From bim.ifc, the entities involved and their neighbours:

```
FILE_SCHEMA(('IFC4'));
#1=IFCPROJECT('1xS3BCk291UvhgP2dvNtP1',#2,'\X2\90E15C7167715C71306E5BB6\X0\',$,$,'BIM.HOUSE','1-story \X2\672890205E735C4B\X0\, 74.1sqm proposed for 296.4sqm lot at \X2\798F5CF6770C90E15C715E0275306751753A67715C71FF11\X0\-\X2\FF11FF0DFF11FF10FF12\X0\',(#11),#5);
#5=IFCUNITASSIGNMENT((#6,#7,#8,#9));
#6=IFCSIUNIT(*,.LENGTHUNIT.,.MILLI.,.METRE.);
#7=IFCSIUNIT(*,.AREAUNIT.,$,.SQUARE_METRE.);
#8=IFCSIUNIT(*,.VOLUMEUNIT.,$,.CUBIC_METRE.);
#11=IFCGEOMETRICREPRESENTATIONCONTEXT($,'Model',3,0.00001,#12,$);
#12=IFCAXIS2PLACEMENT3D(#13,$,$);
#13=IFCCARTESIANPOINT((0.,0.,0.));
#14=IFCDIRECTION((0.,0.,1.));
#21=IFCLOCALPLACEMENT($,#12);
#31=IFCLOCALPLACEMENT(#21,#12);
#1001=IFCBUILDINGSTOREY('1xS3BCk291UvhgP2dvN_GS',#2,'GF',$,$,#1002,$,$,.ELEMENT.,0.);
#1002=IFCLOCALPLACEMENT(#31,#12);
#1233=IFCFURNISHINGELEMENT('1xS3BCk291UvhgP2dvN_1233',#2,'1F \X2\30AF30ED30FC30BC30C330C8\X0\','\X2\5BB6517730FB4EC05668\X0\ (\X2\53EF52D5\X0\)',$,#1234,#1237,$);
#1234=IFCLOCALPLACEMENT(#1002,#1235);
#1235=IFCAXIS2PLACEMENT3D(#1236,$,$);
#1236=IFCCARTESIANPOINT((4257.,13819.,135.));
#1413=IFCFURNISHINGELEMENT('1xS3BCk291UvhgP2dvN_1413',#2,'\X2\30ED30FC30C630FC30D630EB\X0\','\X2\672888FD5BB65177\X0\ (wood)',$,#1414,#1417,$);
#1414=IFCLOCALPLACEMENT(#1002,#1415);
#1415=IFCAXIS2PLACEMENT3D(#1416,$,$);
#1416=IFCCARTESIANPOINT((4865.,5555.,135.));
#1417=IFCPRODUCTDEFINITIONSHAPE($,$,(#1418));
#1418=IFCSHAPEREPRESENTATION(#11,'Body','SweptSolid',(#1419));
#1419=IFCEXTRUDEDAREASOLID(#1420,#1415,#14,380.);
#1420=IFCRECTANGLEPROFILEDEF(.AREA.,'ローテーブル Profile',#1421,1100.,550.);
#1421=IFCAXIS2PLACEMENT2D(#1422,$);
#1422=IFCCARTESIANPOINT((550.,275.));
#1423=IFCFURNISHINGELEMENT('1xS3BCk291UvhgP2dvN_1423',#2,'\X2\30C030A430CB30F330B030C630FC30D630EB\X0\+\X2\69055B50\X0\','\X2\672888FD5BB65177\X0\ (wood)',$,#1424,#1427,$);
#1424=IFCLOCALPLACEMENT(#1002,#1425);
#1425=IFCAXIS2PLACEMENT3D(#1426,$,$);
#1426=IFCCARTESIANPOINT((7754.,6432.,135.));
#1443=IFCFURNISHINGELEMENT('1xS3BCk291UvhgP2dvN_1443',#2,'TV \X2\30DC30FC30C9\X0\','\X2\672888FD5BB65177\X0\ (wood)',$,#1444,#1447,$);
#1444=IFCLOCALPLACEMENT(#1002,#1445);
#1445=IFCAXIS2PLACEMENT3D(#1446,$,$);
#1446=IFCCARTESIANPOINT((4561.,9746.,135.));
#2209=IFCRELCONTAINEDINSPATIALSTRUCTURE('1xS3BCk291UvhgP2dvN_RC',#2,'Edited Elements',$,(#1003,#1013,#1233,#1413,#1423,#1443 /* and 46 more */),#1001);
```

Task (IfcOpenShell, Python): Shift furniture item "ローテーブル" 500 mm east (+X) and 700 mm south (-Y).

```python
import ifcopenshell
import ifcopenshell.api.geometry
import ifcopenshell.util.placement

model = ifcopenshell.open("bim.ifc")

item = model.by_guid("1xS3BCk291UvhgP2dvN_1413")
matrix = ifcopenshell.util.placement.get_local_placement(item.ObjectPlacement)
matrix[0, 3] += 500.0
matrix[1, 3] -= 700.0
ifcopenshell.api.geometry.edit_object_placement(model, product=item, matrix=matrix, is_si=False)

print(ifcopenshell.util.placement.get_local_placement(item.ObjectPlacement).round(3) + 0.0)

model.write("bim-out.ifc")
```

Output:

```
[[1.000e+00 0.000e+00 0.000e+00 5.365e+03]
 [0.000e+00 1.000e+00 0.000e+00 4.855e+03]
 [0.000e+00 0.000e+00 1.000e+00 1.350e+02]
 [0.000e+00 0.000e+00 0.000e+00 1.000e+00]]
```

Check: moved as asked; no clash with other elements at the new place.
